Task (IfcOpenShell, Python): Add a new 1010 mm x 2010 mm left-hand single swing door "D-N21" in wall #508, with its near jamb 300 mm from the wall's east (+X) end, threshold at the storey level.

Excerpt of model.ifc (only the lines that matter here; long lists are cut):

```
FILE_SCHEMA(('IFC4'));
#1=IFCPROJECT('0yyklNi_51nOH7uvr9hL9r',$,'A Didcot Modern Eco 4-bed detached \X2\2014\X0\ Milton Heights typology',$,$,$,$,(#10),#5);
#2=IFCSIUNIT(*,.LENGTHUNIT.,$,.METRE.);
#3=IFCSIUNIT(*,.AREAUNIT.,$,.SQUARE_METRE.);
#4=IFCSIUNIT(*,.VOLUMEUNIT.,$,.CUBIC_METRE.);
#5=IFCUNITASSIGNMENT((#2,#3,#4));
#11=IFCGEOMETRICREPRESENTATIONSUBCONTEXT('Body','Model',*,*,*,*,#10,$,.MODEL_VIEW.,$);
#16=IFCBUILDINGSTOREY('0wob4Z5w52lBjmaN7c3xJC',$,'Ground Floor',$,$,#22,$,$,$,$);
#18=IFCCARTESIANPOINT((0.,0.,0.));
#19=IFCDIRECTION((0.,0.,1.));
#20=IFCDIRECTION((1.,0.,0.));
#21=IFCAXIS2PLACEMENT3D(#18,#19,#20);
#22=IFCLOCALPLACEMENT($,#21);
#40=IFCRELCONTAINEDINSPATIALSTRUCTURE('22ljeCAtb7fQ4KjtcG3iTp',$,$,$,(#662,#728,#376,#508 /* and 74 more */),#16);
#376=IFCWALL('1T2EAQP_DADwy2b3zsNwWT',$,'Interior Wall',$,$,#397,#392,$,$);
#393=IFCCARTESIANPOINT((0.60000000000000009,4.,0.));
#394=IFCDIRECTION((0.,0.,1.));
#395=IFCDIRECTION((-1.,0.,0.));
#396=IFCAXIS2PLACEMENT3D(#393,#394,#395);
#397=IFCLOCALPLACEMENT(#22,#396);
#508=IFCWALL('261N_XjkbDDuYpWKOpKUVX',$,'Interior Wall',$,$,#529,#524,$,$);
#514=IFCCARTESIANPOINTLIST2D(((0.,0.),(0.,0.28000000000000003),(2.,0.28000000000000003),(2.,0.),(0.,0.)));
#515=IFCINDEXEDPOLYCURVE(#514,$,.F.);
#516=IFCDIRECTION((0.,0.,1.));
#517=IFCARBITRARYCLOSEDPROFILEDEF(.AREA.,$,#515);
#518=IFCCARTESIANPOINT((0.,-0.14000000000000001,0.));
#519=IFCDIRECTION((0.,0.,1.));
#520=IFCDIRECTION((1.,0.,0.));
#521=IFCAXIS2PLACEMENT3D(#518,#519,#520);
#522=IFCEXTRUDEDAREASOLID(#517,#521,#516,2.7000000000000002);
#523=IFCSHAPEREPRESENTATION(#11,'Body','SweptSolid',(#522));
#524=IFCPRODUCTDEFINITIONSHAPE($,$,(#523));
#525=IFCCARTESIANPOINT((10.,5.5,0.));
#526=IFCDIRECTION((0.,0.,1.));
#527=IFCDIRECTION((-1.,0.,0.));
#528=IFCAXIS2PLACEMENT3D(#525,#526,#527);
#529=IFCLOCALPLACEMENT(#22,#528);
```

```python
import numpy as np
import ifcopenshell
import ifcopenshell.api.feature
import ifcopenshell.api.geometry
import ifcopenshell.api.root
import ifcopenshell.api.spatial
import ifcopenshell.geom
import ifcopenshell.util.element
import ifcopenshell.util.placement
import ifcopenshell.util.representation
import ifcopenshell.util.shape
import ifcopenshell.util.unit

model = ifcopenshell.open("model.ifc")
unit_scale = ifcopenshell.util.unit.calculate_unit_scale(model)
settings = ifcopenshell.geom.settings()


def volume(element):
    """Net volume in cubic metres, openings subtracted."""
    shape = ifcopenshell.geom.create_shape(settings, element)
    return ifcopenshell.util.shape.get_volume(shape.geometry)


wall = model.by_guid("261N_XjkbDDuYpWKOpKUVX")
storey = ifcopenshell.util.element.get_container(wall, ifc_class="IfcBuildingStorey")
context = ifcopenshell.util.representation.get_context(model, "Model", "Body", "MODEL_VIEW")
before = volume(wall)

width, height, from_end, sill = 1.01, 2.01, 0.3, 0.0  # metres

# The wall runs along its own X axis, and the end named is its -X end.
wall_shape = ifcopenshell.geom.create_shape(settings, wall)
x, y, z = ifcopenshell.util.shape.get_vertices(wall_shape.geometry).T
start = x.min() + from_end
face, thickness = float(y.min()), float(y.max() - y.min())
wall_matrix = ifcopenshell.util.placement.get_local_placement(wall.ObjectPlacement)
level = ifcopenshell.util.placement.get_local_placement(storey.ObjectPlacement)[2, 3]


def in_wall(x, y):
    """Placement at x, y metres in the wall's axes, at sill height."""
    matrix = wall_matrix.copy()
    matrix[:, 3] = wall_matrix @ np.array([x / unit_scale, y / unit_scale, 0.0, 1.0])
    matrix[2, 3] = level + sill / unit_scale
    return matrix


# Opening: a box that overshoots both wall faces by 50 mm.
opening = ifcopenshell.api.root.create_entity(model, ifc_class="IfcOpeningElement", predefined_type="OPENING")
box = ifcopenshell.api.geometry.add_wall_representation(
    model, context=context, length=width, height=height, thickness=thickness + 0.1
)
ifcopenshell.api.geometry.assign_representation(model, product=opening, representation=box)
ifcopenshell.api.geometry.edit_object_placement(model, product=opening, matrix=in_wall(start, face - 0.05), is_si=False)
ifcopenshell.api.feature.add_feature(model, feature=opening, element=wall)

door = ifcopenshell.api.root.create_entity(model, ifc_class="IfcDoor", name="D-N21", predefined_type="DOOR")
door.OverallWidth, door.OverallHeight = width / unit_scale, height / unit_scale
door.OperationType = "SINGLE_SWING_LEFT"
body = ifcopenshell.api.geometry.add_door_representation(
    model,
    context=context,
    overall_width=door.OverallWidth,
    overall_height=door.OverallHeight,
    operation_type="SINGLE_SWING_LEFT",
    lining_properties={"LiningDepth": thickness / unit_scale, "ThresholdDepth": thickness / unit_scale},
)
ifcopenshell.api.geometry.assign_representation(model, product=door, representation=body)
ifcopenshell.api.spatial.assign_container(model, products=[door], relating_structure=storey)
ifcopenshell.api.feature.add_filling(model, opening=opening, element=door)

# The lining spans the wall, so the door starts at the wall face.
ifcopenshell.api.geometry.edit_object_placement(model, product=door, matrix=in_wall(start, face), is_si=False)

after = volume(wall)

print(f"wall volume {before:.3f} -> {after:.3f} m3")

model.write("model_updated.ifc")
```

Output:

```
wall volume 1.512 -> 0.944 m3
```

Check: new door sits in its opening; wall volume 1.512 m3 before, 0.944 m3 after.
